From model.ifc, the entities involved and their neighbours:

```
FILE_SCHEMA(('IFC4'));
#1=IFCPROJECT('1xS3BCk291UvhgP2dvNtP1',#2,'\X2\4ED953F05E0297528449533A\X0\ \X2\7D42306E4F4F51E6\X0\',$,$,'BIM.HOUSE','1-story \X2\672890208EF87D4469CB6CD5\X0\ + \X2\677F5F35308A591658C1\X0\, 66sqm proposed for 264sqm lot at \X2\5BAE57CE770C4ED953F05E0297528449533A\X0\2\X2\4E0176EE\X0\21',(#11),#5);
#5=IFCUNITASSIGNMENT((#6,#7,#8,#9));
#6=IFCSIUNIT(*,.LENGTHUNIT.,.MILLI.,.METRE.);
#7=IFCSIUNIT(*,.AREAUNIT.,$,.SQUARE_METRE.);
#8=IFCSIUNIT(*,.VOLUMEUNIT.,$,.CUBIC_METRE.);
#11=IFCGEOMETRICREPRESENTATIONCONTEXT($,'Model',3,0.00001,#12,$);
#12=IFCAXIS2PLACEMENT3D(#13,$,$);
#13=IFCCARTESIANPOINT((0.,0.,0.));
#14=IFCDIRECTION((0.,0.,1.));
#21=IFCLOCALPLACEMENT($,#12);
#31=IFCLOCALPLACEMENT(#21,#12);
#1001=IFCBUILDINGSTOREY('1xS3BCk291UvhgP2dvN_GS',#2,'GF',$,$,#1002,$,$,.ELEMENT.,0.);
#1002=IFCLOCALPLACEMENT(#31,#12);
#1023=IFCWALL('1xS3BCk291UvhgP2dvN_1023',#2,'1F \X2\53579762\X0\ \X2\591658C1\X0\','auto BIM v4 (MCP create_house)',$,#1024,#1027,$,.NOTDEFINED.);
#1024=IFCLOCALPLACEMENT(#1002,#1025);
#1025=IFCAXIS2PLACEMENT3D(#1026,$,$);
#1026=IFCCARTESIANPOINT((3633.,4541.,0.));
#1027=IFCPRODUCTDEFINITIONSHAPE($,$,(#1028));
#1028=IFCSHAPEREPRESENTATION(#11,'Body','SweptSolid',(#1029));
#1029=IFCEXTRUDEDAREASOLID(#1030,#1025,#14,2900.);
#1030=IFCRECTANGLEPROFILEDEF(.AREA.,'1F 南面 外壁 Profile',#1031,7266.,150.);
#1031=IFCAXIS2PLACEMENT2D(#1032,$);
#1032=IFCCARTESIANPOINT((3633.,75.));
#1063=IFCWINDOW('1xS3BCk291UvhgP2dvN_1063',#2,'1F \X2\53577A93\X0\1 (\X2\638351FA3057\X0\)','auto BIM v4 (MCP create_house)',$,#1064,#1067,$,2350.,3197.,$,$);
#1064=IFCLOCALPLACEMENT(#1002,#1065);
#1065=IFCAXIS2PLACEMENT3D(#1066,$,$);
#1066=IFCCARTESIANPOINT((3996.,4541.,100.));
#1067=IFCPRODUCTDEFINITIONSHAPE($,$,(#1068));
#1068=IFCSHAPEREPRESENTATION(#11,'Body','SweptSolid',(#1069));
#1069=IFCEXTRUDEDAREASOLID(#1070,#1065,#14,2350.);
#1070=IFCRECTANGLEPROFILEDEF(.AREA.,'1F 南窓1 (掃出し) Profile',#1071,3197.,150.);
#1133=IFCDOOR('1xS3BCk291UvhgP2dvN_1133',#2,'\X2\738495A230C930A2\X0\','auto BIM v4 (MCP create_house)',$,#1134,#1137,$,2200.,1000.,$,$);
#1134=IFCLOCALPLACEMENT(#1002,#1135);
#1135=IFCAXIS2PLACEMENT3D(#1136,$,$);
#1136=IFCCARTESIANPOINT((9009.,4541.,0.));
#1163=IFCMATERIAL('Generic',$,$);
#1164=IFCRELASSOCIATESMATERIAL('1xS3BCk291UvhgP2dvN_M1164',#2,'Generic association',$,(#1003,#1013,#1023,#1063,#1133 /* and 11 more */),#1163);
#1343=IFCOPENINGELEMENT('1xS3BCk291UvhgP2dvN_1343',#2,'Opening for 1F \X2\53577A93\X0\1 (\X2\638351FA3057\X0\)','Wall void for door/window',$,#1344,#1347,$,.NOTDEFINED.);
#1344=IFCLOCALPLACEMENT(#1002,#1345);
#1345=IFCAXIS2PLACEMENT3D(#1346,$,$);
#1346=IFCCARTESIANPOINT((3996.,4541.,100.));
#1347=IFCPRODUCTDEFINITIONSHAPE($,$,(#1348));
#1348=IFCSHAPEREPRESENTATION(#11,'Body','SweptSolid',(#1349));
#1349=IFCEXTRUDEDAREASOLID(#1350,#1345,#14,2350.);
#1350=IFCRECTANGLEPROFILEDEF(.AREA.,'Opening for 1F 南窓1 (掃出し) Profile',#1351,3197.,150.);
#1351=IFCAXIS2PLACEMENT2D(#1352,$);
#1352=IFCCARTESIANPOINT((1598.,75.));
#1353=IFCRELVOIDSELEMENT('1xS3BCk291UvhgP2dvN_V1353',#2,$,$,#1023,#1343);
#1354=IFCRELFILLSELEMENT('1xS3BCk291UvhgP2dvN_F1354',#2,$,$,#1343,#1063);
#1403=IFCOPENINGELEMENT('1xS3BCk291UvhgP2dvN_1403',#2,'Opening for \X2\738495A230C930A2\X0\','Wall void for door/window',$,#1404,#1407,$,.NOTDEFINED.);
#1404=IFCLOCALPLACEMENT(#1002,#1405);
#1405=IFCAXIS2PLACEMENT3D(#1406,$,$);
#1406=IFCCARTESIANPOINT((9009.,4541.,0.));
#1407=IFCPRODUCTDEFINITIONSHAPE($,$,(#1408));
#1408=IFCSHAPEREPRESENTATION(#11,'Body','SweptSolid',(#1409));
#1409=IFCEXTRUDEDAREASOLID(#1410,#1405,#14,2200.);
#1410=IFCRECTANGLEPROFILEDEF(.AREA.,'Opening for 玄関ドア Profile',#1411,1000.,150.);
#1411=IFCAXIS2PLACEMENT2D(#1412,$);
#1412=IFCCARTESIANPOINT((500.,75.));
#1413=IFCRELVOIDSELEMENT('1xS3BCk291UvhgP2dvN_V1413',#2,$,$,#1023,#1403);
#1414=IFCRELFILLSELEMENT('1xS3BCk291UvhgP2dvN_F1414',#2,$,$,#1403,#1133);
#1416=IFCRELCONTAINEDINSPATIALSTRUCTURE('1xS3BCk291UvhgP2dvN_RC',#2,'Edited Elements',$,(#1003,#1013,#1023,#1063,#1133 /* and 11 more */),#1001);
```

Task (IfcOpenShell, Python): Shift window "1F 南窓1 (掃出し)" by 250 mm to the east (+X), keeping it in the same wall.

```python
import ifcopenshell
import ifcopenshell.api.geometry
import ifcopenshell.util.placement

model = ifcopenshell.open("model.ifc")

window = model.by_id(1063)
opening = window.FillsVoids[0].RelatingOpeningElement
wall = opening.VoidsElements[0].RelatingBuildingElement

wall_matrix = ifcopenshell.util.placement.get_local_placement(wall.ObjectPlacement)
shift = wall_matrix[:3, 0] * 250.0
before = ifcopenshell.util.placement.get_local_placement(window.ObjectPlacement)[:3, 3].copy()

# The window is not placed relative to its opening, so move both.
for product in (opening, window):
    matrix = ifcopenshell.util.placement.get_local_placement(product.ObjectPlacement)
    matrix[:3, 3] += shift
    ifcopenshell.api.geometry.edit_object_placement(model, product=product, matrix=matrix, is_si=False)

after = ifcopenshell.util.placement.get_local_placement(window.ObjectPlacement)[:3, 3]
print("window moved by", (after - before).round(3) + 0.0)

model.write("model_v2.ifc")
```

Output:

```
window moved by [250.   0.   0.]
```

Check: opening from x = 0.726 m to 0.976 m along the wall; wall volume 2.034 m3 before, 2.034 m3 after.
